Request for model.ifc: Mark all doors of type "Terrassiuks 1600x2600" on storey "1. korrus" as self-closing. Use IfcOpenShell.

First a look at what the model holds.

```python
import ifcopenshell
import ifcopenshell.util.element

model = ifcopenshell.open("model.ifc")
print(model.schema)
storey = next(s for s in model.by_type("IfcBuildingStorey") if s.Name == "1. korrus")
doors = [e for e in ifcopenshell.util.element.get_decomposition(storey) if e.is_a("IfcDoor")]
seen = {}
for e in doors:
    element_type = ifcopenshell.util.element.get_type(e)
    key = (element_type.Name if element_type != e and element_type else None, ifcopenshell.util.element.get_pset(e, "Pset_DoorCommon", "SelfClosing"))
    seen[key] = seen.get(key, 0) + 1
for (name, value), count in sorted(seen.items(), key=str):
    print(count, "x", name, "|", value)
```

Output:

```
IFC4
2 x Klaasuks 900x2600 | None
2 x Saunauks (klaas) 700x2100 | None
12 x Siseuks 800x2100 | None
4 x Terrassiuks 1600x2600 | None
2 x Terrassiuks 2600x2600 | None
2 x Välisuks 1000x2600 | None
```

```python
import ifcopenshell
import ifcopenshell.api.pset
import ifcopenshell.util.element

model = ifcopenshell.open("model.ifc")

storey = next(s for s in model.by_type("IfcBuildingStorey") if s.Name == "1. korrus")
doors = [e for e in ifcopenshell.util.element.get_decomposition(storey) if e.is_a("IfcDoor")]

count = 0
for e in doors:
    element_type = ifcopenshell.util.element.get_type(e)
    if element_type in (None, e) or element_type.Name != "Terrassiuks 1600x2600":
        continue
    # add_pset returns the element's existing set when there is one.
    pset = ifcopenshell.api.pset.add_pset(model, product=e, name="Pset_DoorCommon")
    ifcopenshell.api.pset.edit_pset(model, pset=pset, properties={"SelfClosing": True})
    count += 1

print(count, "doors updated")

model.write("model_rev.ifc")
```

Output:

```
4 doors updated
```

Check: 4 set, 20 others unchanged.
